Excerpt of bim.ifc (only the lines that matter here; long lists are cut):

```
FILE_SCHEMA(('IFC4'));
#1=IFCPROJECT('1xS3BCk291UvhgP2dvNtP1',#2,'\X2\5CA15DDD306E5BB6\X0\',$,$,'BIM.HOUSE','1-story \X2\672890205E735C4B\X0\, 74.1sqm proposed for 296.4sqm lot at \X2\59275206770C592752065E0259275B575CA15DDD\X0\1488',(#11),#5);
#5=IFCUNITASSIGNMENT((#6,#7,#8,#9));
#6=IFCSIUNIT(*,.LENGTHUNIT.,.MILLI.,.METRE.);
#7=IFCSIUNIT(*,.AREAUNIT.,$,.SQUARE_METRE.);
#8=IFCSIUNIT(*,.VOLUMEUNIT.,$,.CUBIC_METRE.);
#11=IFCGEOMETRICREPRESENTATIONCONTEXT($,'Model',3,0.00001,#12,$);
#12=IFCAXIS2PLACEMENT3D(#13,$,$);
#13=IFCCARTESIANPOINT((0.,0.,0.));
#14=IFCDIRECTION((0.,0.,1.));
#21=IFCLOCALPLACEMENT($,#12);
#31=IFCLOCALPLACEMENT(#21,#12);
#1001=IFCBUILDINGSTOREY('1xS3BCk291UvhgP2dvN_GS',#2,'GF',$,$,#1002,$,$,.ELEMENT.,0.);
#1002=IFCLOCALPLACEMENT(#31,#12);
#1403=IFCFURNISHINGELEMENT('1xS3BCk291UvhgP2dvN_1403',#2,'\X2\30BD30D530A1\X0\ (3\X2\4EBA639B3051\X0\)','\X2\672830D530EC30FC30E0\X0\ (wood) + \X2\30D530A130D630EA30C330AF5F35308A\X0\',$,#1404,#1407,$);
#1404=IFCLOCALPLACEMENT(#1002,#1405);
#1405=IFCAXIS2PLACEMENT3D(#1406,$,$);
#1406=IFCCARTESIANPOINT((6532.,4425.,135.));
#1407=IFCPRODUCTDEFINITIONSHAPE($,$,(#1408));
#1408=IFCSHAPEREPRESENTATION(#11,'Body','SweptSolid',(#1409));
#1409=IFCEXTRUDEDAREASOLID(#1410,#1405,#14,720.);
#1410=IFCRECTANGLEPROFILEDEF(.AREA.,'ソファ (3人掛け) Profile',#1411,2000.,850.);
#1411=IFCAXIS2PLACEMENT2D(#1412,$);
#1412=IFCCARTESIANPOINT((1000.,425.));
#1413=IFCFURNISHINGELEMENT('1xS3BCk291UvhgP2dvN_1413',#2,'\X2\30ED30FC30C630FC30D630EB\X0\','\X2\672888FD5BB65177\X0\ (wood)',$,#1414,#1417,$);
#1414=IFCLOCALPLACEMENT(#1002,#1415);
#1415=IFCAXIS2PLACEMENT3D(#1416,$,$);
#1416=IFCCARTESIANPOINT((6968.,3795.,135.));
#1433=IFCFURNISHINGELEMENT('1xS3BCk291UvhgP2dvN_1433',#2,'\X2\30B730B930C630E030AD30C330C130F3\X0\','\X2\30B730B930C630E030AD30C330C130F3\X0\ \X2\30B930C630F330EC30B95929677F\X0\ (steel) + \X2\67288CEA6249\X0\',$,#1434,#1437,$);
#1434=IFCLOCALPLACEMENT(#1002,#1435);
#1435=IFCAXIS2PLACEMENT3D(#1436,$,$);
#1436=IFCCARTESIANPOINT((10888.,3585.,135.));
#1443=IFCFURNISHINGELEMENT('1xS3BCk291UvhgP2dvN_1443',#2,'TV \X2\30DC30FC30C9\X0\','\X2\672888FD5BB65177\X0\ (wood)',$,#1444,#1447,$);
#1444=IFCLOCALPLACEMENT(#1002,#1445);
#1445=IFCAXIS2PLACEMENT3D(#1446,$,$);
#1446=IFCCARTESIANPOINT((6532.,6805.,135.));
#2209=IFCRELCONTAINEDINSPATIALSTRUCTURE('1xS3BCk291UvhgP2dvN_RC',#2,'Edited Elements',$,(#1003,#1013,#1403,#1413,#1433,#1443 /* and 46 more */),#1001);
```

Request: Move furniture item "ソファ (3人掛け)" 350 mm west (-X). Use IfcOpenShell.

```python
import ifcopenshell
import ifcopenshell.api.geometry
import ifcopenshell.util.placement

model = ifcopenshell.open("bim.ifc")

item = model.by_id(1403)
matrix = ifcopenshell.util.placement.get_local_placement(item.ObjectPlacement)
matrix[0, 3] -= 350.0
ifcopenshell.api.geometry.edit_object_placement(model, product=item, matrix=matrix, is_si=False)

print(ifcopenshell.util.placement.get_local_placement(item.ObjectPlacement).round(3) + 0.0)

model.write("bim-out.ifc")
```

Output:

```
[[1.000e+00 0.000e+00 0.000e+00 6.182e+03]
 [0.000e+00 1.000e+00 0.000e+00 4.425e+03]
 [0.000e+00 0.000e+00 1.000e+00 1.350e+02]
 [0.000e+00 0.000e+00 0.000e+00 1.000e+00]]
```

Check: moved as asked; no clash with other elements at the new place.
